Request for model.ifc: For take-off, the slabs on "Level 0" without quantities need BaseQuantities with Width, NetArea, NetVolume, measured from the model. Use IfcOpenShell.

First a look at what the model holds.

```python
import ifcopenshell
import ifcopenshell.util.element
import ifcopenshell.util.unit

model = ifcopenshell.open("model.ifc")
print(model.schema)
for unit_type in ("LENGTHUNIT", "AREAUNIT", "VOLUMEUNIT"):
    print(unit_type, ifcopenshell.util.unit.calculate_unit_scale(model, unit_type))
storey = next(s for s in model.by_type("IfcBuildingStorey") if s.Name == "Level 0")
slabs = [e for e in ifcopenshell.util.element.get_decomposition(storey) if e.is_a("IfcSlab")]
for e in sorted(slabs, key=lambda e: e.id()):
    print(e.id(), e.is_a(), e.Name, list(ifcopenshell.util.element.get_psets(e, qtos_only=True)), sep=" | ")
```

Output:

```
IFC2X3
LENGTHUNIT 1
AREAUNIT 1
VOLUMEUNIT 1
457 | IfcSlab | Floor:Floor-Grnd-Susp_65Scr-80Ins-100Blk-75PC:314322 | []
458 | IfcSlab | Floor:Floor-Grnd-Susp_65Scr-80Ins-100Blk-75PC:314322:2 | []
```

```python
import ifcopenshell
import ifcopenshell.api.pset
import ifcopenshell.geom
import ifcopenshell.util.element
import ifcopenshell.util.shape
import ifcopenshell.util.unit

model = ifcopenshell.open("model.ifc")
unit_scale = ifcopenshell.util.unit.calculate_unit_scale(model)
area_scale = ifcopenshell.util.unit.calculate_unit_scale(model, "AREAUNIT")
volume_scale = ifcopenshell.util.unit.calculate_unit_scale(model, "VOLUMEUNIT")
settings = ifcopenshell.geom.settings()

storey = next(s for s in model.by_type("IfcBuildingStorey") if s.Name == "Level 0")
slabs = [e for e in ifcopenshell.util.element.get_decomposition(storey) if e.is_a("IfcSlab")]

for e in sorted(slabs, key=lambda e: e.id()):
    if ifcopenshell.util.element.get_psets(e, qtos_only=True, should_inherit=False):
        continue
    # Geometry comes back in metres, in the element's own axes.
    shape = ifcopenshell.geom.create_shape(settings, e)
    values = {
        "Width": ifcopenshell.util.shape.get_z(shape.geometry) / unit_scale,
        "NetArea": ifcopenshell.util.shape.get_footprint_area(shape.geometry) / area_scale,
        "NetVolume": ifcopenshell.util.shape.get_volume(shape.geometry) / volume_scale,
    }
    qto = ifcopenshell.api.pset.add_qto(model, product=e, name="BaseQuantities")
    ifcopenshell.api.pset.edit_qto(model, qto=qto, properties=values)
    print(e.id(), {k: round(v, 3) for k, v in values.items()})

model.write("model_edited.ifc")
```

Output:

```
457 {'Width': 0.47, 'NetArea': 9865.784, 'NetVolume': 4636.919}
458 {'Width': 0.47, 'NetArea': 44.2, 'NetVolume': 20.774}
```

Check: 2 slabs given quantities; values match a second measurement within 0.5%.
